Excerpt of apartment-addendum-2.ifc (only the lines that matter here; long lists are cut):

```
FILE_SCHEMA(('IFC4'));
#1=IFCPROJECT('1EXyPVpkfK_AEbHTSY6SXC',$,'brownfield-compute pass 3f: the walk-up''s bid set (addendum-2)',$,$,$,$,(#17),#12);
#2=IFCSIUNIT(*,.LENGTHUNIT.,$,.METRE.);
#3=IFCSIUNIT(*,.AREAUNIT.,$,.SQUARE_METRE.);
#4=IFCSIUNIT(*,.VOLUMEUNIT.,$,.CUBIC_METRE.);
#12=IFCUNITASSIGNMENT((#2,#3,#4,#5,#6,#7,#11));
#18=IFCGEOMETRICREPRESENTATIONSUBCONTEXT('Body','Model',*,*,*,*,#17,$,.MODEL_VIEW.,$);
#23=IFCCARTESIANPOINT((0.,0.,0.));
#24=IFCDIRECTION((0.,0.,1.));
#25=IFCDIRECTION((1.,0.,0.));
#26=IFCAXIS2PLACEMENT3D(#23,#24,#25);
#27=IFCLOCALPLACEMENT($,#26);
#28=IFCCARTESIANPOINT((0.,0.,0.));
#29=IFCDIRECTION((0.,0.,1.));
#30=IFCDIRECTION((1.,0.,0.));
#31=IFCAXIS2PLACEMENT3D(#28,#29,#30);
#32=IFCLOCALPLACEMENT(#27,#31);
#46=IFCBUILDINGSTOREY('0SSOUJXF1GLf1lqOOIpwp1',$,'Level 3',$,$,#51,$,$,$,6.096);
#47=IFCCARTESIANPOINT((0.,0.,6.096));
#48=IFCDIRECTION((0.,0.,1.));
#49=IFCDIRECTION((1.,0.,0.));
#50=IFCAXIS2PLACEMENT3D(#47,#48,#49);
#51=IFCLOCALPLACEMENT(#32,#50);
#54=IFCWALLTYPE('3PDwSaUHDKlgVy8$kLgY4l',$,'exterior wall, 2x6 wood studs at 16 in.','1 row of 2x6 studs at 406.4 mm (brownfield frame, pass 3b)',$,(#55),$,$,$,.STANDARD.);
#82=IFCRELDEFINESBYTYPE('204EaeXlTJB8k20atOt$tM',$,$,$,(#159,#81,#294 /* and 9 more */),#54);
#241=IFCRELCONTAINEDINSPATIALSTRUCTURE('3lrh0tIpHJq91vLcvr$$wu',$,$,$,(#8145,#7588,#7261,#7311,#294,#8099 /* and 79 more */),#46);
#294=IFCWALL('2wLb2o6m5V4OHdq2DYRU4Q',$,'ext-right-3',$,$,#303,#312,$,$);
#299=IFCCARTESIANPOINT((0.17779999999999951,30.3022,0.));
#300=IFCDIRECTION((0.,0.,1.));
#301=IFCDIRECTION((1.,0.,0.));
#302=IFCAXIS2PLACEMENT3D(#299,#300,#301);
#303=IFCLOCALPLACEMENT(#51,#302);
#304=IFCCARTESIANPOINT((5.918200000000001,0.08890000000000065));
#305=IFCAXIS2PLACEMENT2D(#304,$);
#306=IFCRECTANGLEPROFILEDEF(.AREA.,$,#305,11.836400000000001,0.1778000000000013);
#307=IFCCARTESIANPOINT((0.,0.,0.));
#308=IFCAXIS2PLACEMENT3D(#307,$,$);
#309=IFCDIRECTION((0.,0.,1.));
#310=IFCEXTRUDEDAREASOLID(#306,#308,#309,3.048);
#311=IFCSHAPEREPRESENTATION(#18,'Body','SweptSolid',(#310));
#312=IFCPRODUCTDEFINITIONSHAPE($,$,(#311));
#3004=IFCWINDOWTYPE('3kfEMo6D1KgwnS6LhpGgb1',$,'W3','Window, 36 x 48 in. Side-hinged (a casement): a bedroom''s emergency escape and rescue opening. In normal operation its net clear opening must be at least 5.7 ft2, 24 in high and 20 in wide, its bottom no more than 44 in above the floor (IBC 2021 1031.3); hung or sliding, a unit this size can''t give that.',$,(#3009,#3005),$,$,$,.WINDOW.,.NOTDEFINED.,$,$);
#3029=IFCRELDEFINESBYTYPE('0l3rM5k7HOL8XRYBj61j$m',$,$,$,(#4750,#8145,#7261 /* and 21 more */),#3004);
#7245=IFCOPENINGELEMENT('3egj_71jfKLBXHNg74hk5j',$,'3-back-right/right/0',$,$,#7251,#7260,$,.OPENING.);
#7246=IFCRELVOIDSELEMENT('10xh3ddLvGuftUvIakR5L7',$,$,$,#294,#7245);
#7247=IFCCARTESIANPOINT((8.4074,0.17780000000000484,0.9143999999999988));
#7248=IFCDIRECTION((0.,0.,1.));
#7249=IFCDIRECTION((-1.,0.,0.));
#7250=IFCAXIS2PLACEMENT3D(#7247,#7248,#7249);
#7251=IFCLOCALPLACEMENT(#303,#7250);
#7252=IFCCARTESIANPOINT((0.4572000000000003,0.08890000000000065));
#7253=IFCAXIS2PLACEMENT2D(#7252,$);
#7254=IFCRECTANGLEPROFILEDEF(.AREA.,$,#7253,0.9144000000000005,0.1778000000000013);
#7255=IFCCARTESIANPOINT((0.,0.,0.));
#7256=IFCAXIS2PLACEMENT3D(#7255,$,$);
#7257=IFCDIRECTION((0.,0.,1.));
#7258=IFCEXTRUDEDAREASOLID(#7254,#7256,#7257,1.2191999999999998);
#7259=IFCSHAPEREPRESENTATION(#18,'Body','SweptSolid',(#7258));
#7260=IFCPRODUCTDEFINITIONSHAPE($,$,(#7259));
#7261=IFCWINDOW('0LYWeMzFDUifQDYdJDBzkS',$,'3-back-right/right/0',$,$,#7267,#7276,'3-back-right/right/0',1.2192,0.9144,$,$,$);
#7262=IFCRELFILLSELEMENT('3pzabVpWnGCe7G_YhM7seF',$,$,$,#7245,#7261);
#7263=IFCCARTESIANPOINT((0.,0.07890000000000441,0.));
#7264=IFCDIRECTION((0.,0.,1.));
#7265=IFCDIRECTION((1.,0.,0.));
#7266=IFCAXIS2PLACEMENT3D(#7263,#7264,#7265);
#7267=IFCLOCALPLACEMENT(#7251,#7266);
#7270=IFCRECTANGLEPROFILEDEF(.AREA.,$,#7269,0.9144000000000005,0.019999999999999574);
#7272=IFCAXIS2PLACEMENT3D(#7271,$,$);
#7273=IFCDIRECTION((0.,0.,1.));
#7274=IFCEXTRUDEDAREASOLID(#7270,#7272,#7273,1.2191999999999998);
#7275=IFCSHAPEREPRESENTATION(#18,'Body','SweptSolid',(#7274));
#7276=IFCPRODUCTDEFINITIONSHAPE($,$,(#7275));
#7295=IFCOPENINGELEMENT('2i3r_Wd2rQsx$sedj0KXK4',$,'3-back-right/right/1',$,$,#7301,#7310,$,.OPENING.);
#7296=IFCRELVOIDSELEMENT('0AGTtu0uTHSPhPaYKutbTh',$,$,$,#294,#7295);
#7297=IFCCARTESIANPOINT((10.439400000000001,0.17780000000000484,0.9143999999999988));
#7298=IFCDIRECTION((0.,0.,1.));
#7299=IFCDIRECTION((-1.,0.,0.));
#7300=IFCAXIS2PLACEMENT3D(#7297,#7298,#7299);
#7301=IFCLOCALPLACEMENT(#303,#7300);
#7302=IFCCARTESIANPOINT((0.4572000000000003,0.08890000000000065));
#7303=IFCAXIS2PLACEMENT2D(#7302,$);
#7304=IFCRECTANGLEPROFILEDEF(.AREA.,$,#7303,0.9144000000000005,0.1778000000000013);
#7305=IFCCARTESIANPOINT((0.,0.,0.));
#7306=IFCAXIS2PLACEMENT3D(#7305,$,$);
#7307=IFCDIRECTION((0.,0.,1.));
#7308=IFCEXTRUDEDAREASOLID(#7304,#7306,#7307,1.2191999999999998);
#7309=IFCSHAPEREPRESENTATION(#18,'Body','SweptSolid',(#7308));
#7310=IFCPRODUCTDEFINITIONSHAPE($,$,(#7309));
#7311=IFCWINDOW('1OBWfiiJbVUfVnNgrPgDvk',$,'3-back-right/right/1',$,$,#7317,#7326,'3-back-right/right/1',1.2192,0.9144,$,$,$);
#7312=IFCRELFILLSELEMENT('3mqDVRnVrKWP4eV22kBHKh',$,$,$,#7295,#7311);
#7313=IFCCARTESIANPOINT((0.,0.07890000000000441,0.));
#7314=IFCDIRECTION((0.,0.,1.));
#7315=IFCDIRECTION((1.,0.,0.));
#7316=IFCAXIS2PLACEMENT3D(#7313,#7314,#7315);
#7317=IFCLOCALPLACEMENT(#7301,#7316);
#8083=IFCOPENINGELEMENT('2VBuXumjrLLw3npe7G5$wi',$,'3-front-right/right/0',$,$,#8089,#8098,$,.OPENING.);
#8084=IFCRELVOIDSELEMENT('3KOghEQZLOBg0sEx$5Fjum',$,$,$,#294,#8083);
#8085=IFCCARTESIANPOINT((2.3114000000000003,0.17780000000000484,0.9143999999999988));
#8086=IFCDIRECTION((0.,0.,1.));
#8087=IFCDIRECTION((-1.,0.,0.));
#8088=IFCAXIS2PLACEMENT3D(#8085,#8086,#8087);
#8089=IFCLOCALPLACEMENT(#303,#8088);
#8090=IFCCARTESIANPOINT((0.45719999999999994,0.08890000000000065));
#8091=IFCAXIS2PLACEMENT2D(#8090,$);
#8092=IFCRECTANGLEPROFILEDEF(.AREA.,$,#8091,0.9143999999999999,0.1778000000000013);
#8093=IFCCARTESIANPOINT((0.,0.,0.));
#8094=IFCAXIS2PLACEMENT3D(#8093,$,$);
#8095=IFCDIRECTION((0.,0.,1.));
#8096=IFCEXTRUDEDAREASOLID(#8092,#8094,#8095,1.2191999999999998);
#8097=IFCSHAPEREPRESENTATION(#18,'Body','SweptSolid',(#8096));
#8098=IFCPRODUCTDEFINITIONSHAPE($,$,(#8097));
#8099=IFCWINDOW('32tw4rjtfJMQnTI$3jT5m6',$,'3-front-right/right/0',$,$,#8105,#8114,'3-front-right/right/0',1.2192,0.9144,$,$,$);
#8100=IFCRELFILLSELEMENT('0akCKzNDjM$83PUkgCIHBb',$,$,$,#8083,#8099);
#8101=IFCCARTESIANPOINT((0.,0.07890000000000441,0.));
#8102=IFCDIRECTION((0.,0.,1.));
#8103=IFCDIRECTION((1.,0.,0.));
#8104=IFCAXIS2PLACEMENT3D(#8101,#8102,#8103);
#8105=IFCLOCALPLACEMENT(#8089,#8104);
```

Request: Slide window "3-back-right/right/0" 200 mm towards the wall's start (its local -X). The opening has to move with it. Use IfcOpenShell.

```python
import ifcopenshell
import ifcopenshell.api.geometry
import ifcopenshell.util.placement

model = ifcopenshell.open("apartment-addendum-2.ifc")

window = model.by_id(7261)
opening = window.FillsVoids[0].RelatingOpeningElement
wall = opening.VoidsElements[0].RelatingBuildingElement

wall_matrix = ifcopenshell.util.placement.get_local_placement(wall.ObjectPlacement)
shift = wall_matrix[:3, 0] * -0.2
before = ifcopenshell.util.placement.get_local_placement(window.ObjectPlacement)[:3, 3].copy()

# The window is placed relative to its opening, so it follows when the opening moves.
matrix = ifcopenshell.util.placement.get_local_placement(opening.ObjectPlacement)
matrix[:3, 3] += shift
ifcopenshell.api.geometry.edit_object_placement(
    model, product=opening, matrix=matrix, is_si=False, should_transform_children=True
)

after = ifcopenshell.util.placement.get_local_placement(window.ObjectPlacement)[:3, 3]
print("window moved by", (after - before).round(3) + 0.0)

model.write("apartment-addendum-2_rev.ifc")
```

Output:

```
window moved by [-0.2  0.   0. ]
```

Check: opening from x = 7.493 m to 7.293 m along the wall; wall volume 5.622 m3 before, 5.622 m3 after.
